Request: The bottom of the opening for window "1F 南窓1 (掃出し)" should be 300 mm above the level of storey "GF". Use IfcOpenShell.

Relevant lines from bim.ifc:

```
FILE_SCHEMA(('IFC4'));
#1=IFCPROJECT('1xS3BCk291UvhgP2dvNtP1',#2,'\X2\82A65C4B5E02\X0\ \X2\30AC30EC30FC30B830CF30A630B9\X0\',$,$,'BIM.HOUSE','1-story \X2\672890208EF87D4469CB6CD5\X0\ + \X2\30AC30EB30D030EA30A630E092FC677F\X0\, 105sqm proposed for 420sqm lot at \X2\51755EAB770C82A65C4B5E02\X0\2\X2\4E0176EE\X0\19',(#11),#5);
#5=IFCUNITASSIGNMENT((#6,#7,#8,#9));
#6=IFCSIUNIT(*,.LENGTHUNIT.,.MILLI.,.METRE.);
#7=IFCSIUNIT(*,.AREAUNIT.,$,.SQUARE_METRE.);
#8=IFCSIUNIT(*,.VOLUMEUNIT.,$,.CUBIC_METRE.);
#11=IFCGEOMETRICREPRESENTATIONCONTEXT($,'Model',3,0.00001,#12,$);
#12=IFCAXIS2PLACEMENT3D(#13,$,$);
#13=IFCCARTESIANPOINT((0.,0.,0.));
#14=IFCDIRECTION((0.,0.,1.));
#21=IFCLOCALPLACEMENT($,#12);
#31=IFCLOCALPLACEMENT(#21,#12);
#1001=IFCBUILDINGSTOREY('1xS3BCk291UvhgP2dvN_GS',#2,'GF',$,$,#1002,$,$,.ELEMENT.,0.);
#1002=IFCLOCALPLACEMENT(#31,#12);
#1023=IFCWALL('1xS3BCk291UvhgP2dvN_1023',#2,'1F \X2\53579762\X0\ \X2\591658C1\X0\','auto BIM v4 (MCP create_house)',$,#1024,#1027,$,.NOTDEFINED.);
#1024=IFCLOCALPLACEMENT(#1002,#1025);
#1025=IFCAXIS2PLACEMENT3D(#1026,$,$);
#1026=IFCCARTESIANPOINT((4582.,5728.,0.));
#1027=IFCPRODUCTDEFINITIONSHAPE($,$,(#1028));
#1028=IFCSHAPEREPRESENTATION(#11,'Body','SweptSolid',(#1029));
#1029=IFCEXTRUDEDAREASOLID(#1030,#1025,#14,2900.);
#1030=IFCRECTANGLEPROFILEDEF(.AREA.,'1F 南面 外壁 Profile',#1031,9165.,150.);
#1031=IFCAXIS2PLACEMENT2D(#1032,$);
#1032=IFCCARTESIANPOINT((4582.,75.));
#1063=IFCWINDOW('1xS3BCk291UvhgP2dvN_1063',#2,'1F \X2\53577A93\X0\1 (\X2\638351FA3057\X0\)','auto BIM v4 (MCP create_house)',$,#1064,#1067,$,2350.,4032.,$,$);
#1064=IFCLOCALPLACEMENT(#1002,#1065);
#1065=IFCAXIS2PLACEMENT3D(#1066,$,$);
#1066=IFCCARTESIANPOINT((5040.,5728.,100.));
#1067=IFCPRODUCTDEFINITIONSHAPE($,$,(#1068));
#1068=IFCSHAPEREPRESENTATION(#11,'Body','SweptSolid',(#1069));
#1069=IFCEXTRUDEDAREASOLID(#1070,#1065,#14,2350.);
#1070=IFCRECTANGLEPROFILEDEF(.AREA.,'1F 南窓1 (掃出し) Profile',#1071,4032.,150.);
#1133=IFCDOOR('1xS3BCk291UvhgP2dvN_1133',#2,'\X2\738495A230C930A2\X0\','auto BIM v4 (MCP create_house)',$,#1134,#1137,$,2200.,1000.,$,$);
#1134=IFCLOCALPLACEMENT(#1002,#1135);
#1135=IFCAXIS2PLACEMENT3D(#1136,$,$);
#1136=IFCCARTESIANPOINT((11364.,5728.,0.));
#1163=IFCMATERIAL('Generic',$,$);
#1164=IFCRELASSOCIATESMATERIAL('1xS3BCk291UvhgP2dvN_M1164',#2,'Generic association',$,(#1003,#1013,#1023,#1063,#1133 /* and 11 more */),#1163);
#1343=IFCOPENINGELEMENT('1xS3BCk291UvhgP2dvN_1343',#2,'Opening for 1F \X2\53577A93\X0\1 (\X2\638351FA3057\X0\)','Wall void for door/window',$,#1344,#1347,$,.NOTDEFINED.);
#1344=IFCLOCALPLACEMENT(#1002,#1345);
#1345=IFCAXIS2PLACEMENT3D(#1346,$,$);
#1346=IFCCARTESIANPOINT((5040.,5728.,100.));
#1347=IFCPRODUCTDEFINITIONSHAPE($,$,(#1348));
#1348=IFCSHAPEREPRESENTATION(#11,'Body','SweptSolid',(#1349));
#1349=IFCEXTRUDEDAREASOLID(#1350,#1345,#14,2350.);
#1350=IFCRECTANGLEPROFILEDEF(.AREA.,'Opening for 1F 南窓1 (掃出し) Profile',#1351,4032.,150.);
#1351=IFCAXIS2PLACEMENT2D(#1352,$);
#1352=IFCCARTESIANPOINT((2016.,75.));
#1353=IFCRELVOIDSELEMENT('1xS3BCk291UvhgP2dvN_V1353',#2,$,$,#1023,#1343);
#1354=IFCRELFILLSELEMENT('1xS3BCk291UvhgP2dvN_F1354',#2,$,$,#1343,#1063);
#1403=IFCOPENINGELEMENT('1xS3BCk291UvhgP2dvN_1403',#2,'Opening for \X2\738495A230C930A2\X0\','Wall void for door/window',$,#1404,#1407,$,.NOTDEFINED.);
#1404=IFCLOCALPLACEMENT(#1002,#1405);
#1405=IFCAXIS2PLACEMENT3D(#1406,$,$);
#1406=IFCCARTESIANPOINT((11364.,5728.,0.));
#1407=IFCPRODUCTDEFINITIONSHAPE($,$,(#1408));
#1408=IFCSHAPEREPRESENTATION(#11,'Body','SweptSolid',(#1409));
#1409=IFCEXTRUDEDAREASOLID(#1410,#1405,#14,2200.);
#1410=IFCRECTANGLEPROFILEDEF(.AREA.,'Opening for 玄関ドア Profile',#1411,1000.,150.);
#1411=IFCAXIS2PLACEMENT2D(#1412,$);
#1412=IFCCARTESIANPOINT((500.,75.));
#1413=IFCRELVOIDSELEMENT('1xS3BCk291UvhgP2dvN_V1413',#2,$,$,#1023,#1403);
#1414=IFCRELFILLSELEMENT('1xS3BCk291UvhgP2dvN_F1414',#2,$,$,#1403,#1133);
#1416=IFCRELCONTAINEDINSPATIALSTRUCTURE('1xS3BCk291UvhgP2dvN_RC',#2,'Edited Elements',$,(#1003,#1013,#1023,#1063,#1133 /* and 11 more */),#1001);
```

```python
import numpy as np
import ifcopenshell
import ifcopenshell.api.geometry
import ifcopenshell.geom
import ifcopenshell.util.element
import ifcopenshell.util.placement
import ifcopenshell.util.shape
import ifcopenshell.util.unit

model = ifcopenshell.open("bim.ifc")
unit_scale = ifcopenshell.util.unit.calculate_unit_scale(model)

window = model.by_guid("1xS3BCk291UvhgP2dvN_1063")
opening = window.FillsVoids[0].RelatingOpeningElement
storey = ifcopenshell.util.element.get_container(window, ifc_class="IfcBuildingStorey")
level = ifcopenshell.util.placement.get_local_placement(storey.ObjectPlacement)[2, 3]

# The opening's origin need not be at the sill, so measure its lowest point.
shape = ifcopenshell.geom.create_shape(ifcopenshell.geom.settings(), opening)
bottom = ifcopenshell.util.shape.get_shape_bottom_elevation(shape, shape.geometry) / unit_scale
dz = level + 0.3 / unit_scale - bottom

shift = np.array([0.0, 0.0, dz])
# The window is not placed relative to its opening, so move both.
for product in (opening, window):
    matrix = ifcopenshell.util.placement.get_local_placement(product.ObjectPlacement)
    matrix[:3, 3] += shift
    ifcopenshell.api.geometry.edit_object_placement(model, product=product, matrix=matrix, is_si=False)

print(f"moved by {dz * unit_scale:+.3f} m")

model.write("bim_v2.ifc")
```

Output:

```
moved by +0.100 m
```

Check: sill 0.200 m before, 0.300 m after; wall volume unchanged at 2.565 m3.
